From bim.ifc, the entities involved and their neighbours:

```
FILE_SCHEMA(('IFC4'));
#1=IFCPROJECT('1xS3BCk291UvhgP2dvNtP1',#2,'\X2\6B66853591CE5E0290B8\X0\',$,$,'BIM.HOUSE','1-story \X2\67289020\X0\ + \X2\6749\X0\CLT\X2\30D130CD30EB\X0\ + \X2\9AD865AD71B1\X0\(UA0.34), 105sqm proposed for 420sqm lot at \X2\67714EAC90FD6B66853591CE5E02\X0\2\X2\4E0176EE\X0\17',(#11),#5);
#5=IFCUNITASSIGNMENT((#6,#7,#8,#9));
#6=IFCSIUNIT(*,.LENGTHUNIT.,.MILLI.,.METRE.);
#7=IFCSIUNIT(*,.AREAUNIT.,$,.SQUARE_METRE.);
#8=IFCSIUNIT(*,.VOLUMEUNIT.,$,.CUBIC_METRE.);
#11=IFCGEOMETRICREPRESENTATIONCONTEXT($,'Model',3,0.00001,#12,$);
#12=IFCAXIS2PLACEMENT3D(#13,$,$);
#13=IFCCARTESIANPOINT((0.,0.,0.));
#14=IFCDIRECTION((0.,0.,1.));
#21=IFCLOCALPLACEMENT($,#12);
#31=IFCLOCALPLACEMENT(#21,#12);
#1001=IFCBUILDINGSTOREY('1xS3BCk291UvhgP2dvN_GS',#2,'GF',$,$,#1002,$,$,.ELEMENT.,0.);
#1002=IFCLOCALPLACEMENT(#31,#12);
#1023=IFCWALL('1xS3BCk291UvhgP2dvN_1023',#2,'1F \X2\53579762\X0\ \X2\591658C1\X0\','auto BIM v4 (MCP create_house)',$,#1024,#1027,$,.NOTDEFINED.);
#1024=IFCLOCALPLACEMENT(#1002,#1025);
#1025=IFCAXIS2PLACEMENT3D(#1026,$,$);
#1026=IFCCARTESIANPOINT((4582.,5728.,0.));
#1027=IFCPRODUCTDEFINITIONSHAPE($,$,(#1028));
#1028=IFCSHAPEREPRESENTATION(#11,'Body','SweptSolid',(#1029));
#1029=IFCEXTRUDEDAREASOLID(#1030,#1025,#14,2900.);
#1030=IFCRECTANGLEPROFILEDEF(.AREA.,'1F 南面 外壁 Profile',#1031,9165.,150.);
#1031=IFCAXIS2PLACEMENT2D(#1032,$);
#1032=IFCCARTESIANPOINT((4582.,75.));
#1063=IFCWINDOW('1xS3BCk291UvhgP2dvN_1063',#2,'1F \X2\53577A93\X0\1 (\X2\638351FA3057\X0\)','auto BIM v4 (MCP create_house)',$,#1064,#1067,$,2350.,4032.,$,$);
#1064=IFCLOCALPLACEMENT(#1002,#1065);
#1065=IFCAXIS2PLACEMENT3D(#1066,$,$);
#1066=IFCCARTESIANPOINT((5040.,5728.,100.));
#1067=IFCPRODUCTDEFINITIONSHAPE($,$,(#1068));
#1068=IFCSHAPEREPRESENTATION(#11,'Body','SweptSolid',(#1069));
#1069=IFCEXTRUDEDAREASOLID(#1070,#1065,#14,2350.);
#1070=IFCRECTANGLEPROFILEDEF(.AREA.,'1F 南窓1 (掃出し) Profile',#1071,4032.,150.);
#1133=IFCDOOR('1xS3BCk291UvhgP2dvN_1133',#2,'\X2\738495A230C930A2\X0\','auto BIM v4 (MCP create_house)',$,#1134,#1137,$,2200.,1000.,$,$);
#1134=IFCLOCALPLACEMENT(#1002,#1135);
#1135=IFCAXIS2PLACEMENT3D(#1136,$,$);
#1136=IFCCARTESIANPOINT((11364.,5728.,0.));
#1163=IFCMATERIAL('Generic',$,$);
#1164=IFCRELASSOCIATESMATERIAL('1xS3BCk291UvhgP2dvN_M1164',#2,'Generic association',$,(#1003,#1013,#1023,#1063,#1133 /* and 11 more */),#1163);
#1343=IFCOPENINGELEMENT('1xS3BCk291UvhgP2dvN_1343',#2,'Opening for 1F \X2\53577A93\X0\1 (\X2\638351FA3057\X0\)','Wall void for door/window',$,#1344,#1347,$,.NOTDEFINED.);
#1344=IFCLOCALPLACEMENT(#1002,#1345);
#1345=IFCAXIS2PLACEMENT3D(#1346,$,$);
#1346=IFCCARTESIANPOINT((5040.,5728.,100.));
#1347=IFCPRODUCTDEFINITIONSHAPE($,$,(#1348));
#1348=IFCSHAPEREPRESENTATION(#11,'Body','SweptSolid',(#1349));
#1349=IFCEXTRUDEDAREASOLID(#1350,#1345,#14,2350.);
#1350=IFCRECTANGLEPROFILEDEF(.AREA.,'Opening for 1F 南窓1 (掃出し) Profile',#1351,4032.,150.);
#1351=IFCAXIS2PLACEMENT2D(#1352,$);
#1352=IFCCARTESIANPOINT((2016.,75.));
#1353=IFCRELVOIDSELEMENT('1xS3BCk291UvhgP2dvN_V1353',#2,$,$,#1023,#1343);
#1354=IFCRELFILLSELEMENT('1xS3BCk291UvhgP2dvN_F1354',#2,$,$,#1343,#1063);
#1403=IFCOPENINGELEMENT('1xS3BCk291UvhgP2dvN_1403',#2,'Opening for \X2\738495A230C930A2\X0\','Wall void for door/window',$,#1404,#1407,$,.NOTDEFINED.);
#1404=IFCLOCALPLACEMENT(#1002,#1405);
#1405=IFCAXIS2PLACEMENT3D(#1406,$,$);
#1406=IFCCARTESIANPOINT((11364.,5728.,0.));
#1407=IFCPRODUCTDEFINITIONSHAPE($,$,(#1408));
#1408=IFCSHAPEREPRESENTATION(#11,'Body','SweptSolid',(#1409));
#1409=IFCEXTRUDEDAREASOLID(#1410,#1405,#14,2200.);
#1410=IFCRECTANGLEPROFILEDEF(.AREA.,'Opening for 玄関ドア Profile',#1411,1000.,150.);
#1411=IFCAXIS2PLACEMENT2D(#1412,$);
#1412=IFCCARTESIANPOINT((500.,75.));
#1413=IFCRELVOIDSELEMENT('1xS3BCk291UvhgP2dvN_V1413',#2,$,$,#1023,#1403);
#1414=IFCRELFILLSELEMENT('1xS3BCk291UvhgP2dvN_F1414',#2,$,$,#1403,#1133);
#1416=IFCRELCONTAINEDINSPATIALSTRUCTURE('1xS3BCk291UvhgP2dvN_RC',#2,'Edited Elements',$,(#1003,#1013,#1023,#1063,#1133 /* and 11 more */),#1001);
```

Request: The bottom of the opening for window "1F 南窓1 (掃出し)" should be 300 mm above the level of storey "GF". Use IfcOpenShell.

```python
import numpy as np
import ifcopenshell
import ifcopenshell.api.geometry
import ifcopenshell.geom
import ifcopenshell.util.element
import ifcopenshell.util.placement
import ifcopenshell.util.shape
import ifcopenshell.util.unit

model = ifcopenshell.open("bim.ifc")
unit_scale = ifcopenshell.util.unit.calculate_unit_scale(model)

window = model.by_guid("1xS3BCk291UvhgP2dvN_1063")
opening = window.FillsVoids[0].RelatingOpeningElement
storey = ifcopenshell.util.element.get_container(window, ifc_class="IfcBuildingStorey")
level = ifcopenshell.util.placement.get_local_placement(storey.ObjectPlacement)[2, 3]

# The opening's origin need not be at the sill, so measure its lowest point.
shape = ifcopenshell.geom.create_shape(ifcopenshell.geom.settings(), opening)
bottom = ifcopenshell.util.shape.get_shape_bottom_elevation(shape, shape.geometry) / unit_scale
dz = level + 0.3 / unit_scale - bottom

shift = np.array([0.0, 0.0, dz])
# The window is not placed relative to its opening, so move both.
for product in (opening, window):
    matrix = ifcopenshell.util.placement.get_local_placement(product.ObjectPlacement)
    matrix[:3, 3] += shift
    ifcopenshell.api.geometry.edit_object_placement(model, product=product, matrix=matrix, is_si=False)

print(f"moved by {dz * unit_scale:+.3f} m")

model.write("bim-out.ifc")
```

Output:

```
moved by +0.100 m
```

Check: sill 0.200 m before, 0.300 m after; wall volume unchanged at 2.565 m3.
